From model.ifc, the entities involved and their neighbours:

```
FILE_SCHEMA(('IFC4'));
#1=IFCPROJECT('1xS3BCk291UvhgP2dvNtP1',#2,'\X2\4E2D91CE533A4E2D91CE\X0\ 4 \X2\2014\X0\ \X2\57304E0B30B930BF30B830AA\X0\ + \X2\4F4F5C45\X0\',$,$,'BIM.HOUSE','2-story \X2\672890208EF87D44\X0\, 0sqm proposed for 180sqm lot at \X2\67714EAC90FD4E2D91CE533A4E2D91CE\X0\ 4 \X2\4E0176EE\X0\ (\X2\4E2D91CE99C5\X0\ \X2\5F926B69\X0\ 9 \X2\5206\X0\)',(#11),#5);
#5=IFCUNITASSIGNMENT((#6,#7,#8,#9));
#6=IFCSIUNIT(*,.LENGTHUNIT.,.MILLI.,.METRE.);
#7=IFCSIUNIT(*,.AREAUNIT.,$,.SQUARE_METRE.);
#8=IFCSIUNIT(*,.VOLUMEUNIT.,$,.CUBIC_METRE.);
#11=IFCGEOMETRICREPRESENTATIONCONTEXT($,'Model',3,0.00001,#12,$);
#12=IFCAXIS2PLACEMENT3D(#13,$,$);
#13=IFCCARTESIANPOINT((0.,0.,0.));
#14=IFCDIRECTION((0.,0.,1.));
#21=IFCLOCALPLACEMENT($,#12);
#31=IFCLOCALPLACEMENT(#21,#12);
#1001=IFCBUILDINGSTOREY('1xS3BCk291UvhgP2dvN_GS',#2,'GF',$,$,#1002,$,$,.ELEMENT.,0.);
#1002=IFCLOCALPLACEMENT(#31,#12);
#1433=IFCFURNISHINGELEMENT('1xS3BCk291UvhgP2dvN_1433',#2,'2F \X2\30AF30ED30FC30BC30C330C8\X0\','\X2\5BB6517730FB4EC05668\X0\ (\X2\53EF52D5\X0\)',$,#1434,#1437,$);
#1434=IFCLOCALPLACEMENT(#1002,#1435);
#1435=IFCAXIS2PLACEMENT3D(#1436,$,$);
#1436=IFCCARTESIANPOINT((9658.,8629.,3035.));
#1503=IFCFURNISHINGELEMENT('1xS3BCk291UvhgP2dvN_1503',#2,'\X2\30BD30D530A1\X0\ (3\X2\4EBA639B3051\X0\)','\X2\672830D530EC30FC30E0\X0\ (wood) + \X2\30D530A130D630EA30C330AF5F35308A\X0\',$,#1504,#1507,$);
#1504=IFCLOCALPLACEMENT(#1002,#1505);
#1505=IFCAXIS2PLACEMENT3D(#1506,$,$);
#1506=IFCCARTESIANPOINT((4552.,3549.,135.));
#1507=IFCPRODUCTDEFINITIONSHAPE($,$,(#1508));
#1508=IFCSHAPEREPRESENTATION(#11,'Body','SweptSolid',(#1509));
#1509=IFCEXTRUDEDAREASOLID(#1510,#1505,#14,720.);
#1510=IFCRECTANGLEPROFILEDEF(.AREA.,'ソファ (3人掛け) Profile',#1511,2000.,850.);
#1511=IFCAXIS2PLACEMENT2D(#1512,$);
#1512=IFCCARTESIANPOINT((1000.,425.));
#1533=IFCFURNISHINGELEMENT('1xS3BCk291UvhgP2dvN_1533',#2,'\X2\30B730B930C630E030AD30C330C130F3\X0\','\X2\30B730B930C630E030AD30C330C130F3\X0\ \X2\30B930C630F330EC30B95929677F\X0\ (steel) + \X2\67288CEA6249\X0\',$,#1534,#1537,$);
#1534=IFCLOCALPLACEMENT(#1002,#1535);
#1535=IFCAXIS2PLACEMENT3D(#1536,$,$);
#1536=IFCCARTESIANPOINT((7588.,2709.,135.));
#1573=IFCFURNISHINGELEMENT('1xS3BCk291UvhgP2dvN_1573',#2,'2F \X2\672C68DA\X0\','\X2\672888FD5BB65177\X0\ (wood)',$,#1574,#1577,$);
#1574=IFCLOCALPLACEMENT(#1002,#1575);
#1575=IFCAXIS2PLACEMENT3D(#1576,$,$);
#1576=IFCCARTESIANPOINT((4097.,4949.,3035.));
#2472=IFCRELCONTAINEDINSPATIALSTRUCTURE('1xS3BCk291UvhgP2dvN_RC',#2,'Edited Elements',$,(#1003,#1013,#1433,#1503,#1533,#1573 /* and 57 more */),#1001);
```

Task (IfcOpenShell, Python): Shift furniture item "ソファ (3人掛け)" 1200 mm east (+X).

```python
import ifcopenshell
import ifcopenshell.api.geometry
import ifcopenshell.util.placement
import ifcopenshell.util.unit

model = ifcopenshell.open("model.ifc")
unit_scale = ifcopenshell.util.unit.calculate_unit_scale(model)

item = model.by_id(1503)
matrix = ifcopenshell.util.placement.get_local_placement(item.ObjectPlacement)
matrix[0, 3] += 1.2 / unit_scale
ifcopenshell.api.geometry.edit_object_placement(model, product=item, matrix=matrix, is_si=False)

print(ifcopenshell.util.placement.get_local_placement(item.ObjectPlacement).round(3) + 0.0)

model.write("model-out.ifc")
```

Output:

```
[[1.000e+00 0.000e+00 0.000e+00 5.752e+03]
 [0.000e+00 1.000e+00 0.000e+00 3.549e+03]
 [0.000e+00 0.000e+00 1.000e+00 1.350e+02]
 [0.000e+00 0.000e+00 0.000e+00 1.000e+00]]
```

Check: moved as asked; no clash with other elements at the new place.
